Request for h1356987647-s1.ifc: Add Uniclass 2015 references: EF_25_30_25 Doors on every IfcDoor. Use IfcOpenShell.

First a look at what the model holds.

```python
import ifcopenshell

model = ifcopenshell.open("h1356987647-s1.ifc")
print(model.schema)
print("classifications:", [c.Name for c in model.by_type("IfcClassification")])
for ifc_class in ("IfcDoor", "IfcRoof", "IfcStair", "IfcWall", "IfcWindow"):
    print(ifc_class, len(model.by_type(ifc_class)))
```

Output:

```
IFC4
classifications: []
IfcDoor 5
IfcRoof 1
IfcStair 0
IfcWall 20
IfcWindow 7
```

```python
import ifcopenshell
import ifcopenshell.api.classification

model = ifcopenshell.open("h1356987647-s1.ifc")

system = ifcopenshell.api.classification.add_classification(model, classification="Uniclass 2015")

codes = {
    "IfcDoor": ("EF_25_30_25", "Doors"),
}
for ifc_class, (code, name) in codes.items():
    products = model.by_type(ifc_class)
    ifcopenshell.api.classification.add_reference(
        model, products=products, classification=system, identification=code, name=name
    )
    print(code, len(products))

model.write("h1356987647-s1_v2.ifc")
```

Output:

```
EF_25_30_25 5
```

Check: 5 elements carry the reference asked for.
